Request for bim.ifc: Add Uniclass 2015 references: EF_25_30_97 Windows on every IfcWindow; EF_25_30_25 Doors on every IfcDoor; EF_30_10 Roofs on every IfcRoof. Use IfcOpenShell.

First a look at what the model holds.

```python
import ifcopenshell

model = ifcopenshell.open("bim.ifc")
print(model.schema)
print("classifications:", [c.Name for c in model.by_type("IfcClassification")])
for ifc_class in ("IfcDoor", "IfcRoof", "IfcStair", "IfcWall", "IfcWindow"):
    print(ifc_class, len(model.by_type(ifc_class)))
```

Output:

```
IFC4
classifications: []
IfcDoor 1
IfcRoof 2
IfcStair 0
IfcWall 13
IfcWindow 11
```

```python
import ifcopenshell
import ifcopenshell.api.classification

model = ifcopenshell.open("bim.ifc")

system = ifcopenshell.api.classification.add_classification(model, classification="Uniclass 2015")

codes = {
    "IfcWindow": ("EF_25_30_97", "Windows"),
    "IfcDoor": ("EF_25_30_25", "Doors"),
    "IfcRoof": ("EF_30_10", "Roofs"),
}
for ifc_class, (code, name) in codes.items():
    products = model.by_type(ifc_class)
    ifcopenshell.api.classification.add_reference(
        model, products=products, classification=system, identification=code, name=name
    )
    print(code, len(products))

model.write("bim-out.ifc")
```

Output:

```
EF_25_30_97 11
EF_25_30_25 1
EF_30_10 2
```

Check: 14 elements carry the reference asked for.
